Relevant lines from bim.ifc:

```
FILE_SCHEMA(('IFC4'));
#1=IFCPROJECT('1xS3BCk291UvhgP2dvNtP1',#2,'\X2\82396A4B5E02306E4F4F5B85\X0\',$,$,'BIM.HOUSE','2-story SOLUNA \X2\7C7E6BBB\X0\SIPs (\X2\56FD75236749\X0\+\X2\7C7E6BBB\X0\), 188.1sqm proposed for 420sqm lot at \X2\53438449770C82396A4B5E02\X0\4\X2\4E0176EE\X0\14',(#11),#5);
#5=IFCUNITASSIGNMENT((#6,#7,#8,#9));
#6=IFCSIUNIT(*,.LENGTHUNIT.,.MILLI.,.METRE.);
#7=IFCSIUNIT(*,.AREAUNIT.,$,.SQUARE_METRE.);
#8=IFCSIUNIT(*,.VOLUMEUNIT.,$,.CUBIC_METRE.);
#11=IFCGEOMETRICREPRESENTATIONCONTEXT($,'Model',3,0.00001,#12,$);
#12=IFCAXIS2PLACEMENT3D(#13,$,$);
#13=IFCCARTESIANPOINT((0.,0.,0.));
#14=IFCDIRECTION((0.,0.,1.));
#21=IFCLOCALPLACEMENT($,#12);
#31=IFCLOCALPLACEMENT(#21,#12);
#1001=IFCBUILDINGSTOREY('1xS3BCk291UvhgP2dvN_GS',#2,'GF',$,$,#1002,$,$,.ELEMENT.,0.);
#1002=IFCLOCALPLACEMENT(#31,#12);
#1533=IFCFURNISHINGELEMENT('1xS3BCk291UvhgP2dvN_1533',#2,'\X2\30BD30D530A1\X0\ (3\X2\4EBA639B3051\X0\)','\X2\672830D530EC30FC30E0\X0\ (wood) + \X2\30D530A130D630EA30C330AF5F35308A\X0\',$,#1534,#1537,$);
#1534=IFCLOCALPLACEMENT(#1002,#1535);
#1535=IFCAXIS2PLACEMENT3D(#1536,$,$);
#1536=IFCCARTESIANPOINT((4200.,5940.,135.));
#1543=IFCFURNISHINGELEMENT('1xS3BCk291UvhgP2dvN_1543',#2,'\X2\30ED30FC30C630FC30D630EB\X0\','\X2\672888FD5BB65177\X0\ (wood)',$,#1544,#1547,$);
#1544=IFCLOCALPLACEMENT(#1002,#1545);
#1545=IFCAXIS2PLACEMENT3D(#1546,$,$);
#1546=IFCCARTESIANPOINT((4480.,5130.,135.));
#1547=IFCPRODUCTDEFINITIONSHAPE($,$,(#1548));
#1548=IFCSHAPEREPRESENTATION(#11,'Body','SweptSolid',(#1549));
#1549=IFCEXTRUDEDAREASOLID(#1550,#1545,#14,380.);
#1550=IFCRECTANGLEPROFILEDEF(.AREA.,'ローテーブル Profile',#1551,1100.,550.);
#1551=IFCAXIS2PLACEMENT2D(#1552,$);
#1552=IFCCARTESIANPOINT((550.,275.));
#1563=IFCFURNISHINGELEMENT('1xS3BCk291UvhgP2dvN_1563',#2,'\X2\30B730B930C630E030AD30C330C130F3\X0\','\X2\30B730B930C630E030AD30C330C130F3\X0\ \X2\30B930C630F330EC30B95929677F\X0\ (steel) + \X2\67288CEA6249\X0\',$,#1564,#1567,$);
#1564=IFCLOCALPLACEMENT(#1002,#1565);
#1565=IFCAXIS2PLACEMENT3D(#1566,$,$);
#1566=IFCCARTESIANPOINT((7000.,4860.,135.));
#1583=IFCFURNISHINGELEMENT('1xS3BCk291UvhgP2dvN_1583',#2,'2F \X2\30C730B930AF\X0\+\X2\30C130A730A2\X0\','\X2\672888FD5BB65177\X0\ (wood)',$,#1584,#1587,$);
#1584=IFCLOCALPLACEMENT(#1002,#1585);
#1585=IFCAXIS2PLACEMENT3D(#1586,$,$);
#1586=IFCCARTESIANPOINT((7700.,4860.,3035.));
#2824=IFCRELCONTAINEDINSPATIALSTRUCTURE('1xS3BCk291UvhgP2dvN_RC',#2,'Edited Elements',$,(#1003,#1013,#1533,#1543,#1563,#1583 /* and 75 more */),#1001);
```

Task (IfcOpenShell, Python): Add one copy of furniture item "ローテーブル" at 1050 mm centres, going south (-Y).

```python
import numpy as np
import ifcopenshell
import ifcopenshell.api.geometry
import ifcopenshell.api.root
import ifcopenshell.util.element
import ifcopenshell.util.placement
import ifcopenshell.util.unit

model = ifcopenshell.open("bim.ifc")
unit_scale = ifcopenshell.util.unit.calculate_unit_scale(model)


def reuse_history(source, copy):
    """copy_class also copies each property set's owner history, people and application; keep the originals."""
    for rel in copy.IsDefinedBy:
        if rel.is_a("IfcRelDefinesByProperties") and (history := rel.RelatingPropertyDefinition.OwnerHistory):
            rel.RelatingPropertyDefinition.OwnerHistory = source.OwnerHistory
            ifcopenshell.util.element.remove_deep2(model, history)


source = model.by_guid("1xS3BCk291UvhgP2dvN_1543")
base = ifcopenshell.util.placement.get_local_placement(source.ObjectPlacement)
step = np.array([0.0, -1.0, 0.0]) * 1.05 / unit_scale

for i in range(1, 2):
    copy = ifcopenshell.api.root.copy_class(model, product=source)
    copy.Representation = ifcopenshell.util.element.copy_deep(
        model, source.Representation, exclude=["IfcGeometricRepresentationContext", "IfcRepresentationMap"]
    )
    reuse_history(source, copy)
    matrix = base.copy()
    matrix[:3, 3] += i * step
    print("added at", matrix[:3, 3].round(3) + 0.0)
    ifcopenshell.api.geometry.edit_object_placement(model, product=copy, matrix=matrix, is_si=False)

model.write("bim_edited.ifc")
```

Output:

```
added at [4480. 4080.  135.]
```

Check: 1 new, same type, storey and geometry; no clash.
